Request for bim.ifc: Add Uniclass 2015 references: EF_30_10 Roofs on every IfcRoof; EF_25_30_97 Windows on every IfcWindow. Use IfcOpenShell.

First a look at what the model holds.

```python
import ifcopenshell

model = ifcopenshell.open("bim.ifc")
print(model.schema)
print("classifications:", [c.Name for c in model.by_type("IfcClassification")])
for ifc_class in ("IfcDoor", "IfcRoof", "IfcStair", "IfcWall", "IfcWindow"):
    print(ifc_class, len(model.by_type(ifc_class)))
```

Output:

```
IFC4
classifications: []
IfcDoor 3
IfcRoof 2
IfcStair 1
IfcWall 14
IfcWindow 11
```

```python
import ifcopenshell
import ifcopenshell.api.classification

model = ifcopenshell.open("bim.ifc")

system = ifcopenshell.api.classification.add_classification(model, classification="Uniclass 2015")

codes = {
    "IfcRoof": ("EF_30_10", "Roofs"),
    "IfcWindow": ("EF_25_30_97", "Windows"),
}
for ifc_class, (code, name) in codes.items():
    products = model.by_type(ifc_class)
    ifcopenshell.api.classification.add_reference(
        model, products=products, classification=system, identification=code, name=name
    )
    print(code, len(products))

model.write("bim_v2.ifc")
```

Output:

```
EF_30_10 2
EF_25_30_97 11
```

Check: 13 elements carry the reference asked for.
